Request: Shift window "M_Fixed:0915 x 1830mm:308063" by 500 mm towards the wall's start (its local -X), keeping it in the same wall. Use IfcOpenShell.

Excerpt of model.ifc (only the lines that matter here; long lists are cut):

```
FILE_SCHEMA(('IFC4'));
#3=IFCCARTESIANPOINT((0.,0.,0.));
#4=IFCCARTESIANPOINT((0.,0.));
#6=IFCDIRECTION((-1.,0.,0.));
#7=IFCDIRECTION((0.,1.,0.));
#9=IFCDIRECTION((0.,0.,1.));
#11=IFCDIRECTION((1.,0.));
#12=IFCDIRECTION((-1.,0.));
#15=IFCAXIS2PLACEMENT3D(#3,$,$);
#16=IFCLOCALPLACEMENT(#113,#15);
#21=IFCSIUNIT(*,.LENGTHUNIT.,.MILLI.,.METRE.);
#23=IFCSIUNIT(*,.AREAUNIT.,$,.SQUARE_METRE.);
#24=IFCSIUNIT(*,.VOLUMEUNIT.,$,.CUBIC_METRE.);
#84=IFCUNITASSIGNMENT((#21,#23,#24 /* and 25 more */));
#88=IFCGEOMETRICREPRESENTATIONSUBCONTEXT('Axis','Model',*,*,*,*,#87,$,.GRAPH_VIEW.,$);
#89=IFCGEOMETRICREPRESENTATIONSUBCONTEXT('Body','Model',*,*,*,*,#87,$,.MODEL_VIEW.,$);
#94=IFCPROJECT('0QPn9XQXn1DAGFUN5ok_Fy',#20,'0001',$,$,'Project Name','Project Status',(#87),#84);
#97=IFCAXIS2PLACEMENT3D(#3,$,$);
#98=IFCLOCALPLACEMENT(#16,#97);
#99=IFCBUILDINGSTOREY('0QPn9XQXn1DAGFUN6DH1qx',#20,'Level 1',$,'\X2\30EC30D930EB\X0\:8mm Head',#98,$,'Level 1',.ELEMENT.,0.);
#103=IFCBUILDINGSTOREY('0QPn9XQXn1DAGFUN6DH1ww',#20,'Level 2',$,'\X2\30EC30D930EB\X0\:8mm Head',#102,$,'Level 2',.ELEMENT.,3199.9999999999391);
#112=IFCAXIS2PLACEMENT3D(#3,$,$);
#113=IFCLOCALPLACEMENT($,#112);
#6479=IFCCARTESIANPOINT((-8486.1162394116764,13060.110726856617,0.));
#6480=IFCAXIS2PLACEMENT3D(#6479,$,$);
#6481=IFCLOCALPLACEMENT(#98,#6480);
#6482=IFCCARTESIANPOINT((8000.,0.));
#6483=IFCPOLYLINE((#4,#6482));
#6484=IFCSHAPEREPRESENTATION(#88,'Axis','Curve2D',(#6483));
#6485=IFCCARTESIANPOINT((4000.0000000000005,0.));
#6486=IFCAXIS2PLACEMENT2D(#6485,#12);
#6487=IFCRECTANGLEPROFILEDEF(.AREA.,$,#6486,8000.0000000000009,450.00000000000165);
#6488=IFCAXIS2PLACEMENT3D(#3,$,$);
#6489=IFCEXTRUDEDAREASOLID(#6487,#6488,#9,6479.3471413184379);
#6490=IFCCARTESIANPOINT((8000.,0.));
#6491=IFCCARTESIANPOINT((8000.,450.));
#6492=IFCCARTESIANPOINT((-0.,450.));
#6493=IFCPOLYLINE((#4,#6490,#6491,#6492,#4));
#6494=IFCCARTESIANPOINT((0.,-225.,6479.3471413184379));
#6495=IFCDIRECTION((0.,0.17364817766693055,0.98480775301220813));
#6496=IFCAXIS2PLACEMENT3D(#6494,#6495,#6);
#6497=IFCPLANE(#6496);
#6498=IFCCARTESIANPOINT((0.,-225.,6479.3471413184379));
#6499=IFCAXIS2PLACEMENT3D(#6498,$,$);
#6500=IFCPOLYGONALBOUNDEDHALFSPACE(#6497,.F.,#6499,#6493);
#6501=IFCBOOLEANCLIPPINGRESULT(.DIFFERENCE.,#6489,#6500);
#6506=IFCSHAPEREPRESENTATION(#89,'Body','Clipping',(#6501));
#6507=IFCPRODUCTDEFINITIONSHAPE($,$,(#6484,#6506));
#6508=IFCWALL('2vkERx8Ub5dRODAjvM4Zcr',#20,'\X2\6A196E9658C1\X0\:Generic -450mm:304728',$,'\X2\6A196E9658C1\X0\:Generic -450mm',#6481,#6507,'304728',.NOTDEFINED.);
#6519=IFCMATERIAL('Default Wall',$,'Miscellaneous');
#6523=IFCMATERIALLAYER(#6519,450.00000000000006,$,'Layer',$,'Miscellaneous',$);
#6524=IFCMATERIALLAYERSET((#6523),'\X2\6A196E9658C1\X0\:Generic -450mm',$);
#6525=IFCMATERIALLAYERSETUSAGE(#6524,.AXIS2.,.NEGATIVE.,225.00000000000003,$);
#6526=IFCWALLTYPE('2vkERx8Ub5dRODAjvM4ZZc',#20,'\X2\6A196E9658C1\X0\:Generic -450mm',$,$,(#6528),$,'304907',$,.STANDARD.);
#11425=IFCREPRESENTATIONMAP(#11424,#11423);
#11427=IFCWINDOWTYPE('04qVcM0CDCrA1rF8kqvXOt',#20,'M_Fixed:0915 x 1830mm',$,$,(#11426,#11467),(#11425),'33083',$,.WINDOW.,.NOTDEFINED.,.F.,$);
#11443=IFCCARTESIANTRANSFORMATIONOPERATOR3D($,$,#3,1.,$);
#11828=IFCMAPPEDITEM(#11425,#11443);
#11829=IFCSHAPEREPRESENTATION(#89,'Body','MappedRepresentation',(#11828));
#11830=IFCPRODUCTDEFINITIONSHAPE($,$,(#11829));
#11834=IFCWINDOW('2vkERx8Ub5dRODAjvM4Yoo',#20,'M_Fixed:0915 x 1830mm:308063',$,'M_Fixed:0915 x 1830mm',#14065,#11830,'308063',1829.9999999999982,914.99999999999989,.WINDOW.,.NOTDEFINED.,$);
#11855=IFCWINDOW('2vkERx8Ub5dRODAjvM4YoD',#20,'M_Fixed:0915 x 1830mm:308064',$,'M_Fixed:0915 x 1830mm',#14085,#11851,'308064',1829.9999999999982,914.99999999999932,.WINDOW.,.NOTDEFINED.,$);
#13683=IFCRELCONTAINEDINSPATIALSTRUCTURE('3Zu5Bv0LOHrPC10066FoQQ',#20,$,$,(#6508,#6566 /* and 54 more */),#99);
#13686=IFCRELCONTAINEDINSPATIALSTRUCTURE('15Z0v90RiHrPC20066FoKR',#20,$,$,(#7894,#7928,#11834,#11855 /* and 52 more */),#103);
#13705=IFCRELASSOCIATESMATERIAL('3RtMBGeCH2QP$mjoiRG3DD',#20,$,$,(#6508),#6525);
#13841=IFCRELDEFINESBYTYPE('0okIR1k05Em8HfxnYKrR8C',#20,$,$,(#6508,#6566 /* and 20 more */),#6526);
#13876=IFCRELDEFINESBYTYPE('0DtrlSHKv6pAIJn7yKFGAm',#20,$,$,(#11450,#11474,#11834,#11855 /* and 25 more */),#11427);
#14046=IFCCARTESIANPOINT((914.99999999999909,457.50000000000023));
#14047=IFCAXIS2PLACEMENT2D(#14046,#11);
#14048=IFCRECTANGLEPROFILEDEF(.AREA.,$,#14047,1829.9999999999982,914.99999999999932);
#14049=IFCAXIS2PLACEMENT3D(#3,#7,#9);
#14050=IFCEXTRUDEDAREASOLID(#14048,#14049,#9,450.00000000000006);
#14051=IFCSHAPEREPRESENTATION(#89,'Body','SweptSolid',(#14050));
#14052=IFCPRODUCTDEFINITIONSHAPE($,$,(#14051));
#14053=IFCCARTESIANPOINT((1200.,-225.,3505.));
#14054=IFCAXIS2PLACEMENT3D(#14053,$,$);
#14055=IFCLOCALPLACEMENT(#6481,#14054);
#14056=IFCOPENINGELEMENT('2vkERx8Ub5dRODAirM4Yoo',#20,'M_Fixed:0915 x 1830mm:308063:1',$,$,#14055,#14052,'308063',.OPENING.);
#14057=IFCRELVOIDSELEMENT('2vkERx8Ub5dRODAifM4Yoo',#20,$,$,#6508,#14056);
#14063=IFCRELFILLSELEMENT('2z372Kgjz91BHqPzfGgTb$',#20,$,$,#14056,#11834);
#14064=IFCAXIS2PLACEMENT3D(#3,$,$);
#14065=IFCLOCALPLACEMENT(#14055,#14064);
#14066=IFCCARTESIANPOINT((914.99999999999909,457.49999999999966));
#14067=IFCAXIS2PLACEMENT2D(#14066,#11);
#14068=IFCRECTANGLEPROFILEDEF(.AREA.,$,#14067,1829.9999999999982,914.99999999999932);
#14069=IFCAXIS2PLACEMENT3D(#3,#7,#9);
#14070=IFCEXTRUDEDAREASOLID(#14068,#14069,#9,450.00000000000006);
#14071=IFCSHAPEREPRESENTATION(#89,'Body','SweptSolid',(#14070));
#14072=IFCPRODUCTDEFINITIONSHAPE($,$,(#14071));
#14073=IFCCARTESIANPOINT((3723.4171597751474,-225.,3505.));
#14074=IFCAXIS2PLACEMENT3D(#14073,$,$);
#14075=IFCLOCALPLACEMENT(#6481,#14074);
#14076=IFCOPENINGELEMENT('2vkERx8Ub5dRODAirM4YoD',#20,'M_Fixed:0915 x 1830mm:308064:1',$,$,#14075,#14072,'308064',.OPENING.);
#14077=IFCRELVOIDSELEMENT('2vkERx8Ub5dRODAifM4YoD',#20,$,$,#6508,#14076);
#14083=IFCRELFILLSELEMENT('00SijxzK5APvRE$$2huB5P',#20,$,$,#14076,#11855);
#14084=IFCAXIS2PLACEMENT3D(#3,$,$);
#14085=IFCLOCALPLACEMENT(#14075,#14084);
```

```python
import ifcopenshell
import ifcopenshell.api.geometry
import ifcopenshell.util.placement

model = ifcopenshell.open("model.ifc")

window = model.by_id(11834)
opening = window.FillsVoids[0].RelatingOpeningElement
wall = opening.VoidsElements[0].RelatingBuildingElement

wall_matrix = ifcopenshell.util.placement.get_local_placement(wall.ObjectPlacement)
shift = wall_matrix[:3, 0] * -500.0
before = ifcopenshell.util.placement.get_local_placement(window.ObjectPlacement)[:3, 3].copy()

# The window is placed relative to its opening, so it follows when the opening moves.
matrix = ifcopenshell.util.placement.get_local_placement(opening.ObjectPlacement)
matrix[:3, 3] += shift
ifcopenshell.api.geometry.edit_object_placement(
    model, product=opening, matrix=matrix, is_si=False, should_transform_children=True
)

after = ifcopenshell.util.placement.get_local_placement(window.ObjectPlacement)[:3, 3]
print("window moved by", (after - before).round(3) + 0.0)

model.write("model_edited.ifc")
```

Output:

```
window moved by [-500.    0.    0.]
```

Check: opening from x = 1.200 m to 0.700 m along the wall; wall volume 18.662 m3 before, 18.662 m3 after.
